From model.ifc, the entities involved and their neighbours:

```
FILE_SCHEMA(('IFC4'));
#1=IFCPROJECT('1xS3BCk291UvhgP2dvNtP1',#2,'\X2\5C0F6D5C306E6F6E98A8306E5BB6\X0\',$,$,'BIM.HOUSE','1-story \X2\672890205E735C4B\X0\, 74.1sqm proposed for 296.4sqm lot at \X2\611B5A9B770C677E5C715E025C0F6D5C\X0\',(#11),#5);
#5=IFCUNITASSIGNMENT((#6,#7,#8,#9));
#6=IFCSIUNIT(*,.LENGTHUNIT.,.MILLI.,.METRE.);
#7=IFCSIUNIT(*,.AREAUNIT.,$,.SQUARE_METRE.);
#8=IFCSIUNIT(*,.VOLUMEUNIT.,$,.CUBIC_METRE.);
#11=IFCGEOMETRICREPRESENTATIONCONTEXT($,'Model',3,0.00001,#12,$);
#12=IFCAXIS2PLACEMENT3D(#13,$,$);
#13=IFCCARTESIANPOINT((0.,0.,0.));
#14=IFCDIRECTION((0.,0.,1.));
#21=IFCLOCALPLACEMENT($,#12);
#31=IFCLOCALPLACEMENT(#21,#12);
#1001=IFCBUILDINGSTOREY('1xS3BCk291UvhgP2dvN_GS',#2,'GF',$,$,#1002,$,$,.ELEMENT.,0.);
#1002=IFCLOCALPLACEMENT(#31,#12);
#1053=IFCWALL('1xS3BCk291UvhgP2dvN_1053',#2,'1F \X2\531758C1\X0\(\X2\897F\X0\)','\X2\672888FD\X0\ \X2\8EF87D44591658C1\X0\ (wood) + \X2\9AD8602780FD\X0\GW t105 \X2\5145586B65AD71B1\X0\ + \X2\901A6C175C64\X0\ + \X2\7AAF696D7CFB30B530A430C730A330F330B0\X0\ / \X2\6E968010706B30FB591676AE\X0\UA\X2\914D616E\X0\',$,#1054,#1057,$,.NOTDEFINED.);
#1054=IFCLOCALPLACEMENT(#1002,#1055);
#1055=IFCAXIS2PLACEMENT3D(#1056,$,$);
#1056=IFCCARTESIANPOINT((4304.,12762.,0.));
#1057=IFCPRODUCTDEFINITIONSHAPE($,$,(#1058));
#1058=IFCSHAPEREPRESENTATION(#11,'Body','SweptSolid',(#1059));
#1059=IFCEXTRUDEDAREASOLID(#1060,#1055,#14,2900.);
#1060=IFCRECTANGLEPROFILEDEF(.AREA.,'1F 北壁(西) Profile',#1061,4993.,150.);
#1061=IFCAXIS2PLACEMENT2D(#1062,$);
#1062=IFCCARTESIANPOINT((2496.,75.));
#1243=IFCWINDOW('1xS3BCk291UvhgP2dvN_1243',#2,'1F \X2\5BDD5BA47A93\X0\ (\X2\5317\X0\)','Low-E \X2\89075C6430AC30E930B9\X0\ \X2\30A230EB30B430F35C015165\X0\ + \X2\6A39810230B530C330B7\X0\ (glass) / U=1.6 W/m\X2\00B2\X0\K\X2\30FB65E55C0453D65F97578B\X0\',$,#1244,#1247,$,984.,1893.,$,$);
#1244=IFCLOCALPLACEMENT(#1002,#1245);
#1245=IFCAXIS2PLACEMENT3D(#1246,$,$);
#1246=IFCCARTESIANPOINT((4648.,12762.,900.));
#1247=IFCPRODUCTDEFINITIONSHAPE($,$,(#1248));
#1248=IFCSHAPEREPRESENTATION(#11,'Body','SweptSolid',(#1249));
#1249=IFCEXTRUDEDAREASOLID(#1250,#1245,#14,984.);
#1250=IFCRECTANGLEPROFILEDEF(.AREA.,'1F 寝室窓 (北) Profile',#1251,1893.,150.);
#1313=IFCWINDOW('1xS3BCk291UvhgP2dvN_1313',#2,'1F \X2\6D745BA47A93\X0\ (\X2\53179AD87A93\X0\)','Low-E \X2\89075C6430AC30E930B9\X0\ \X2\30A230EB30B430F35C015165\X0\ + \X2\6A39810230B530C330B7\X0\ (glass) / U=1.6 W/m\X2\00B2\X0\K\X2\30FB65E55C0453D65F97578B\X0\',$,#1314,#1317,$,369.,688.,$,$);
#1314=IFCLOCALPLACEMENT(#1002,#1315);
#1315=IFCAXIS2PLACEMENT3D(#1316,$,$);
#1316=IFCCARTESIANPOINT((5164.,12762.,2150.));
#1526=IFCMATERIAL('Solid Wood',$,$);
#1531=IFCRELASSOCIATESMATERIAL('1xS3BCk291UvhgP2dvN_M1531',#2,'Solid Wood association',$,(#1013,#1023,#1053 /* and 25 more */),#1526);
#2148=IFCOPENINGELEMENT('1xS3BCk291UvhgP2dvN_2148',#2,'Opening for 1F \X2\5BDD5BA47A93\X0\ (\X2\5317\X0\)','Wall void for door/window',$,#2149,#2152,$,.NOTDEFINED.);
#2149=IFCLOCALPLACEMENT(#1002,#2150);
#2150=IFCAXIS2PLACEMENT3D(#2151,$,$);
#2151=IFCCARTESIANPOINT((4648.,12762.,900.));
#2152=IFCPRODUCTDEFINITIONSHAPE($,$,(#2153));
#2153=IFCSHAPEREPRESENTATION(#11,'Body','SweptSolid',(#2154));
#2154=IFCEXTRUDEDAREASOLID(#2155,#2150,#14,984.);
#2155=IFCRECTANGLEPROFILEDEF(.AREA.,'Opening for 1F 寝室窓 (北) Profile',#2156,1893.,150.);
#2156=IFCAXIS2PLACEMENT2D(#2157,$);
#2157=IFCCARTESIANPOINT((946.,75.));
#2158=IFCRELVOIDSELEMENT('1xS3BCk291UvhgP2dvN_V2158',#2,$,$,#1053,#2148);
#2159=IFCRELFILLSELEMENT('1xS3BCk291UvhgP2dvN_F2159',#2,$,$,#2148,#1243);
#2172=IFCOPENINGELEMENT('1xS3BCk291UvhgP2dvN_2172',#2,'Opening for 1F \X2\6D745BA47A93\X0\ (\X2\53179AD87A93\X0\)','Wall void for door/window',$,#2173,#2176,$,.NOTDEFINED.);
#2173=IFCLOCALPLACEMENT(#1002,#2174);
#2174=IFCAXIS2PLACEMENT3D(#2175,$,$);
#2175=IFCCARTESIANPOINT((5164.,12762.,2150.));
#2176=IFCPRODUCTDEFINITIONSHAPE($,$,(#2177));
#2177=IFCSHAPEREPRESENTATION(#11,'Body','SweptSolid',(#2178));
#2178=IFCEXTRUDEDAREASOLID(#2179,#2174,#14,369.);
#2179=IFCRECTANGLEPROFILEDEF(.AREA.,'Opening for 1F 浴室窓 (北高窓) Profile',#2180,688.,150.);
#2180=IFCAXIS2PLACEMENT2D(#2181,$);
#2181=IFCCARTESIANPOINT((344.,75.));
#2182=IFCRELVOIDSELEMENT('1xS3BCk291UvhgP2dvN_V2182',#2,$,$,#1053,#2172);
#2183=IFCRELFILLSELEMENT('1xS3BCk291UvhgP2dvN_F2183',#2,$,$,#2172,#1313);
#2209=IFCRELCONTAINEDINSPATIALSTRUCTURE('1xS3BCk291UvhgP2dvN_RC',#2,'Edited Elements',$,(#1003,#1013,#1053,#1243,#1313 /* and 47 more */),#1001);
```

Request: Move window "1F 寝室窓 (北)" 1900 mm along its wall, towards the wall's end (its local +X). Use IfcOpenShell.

```python
import ifcopenshell
import ifcopenshell.api.geometry
import ifcopenshell.util.placement

model = ifcopenshell.open("model.ifc")

window = model.by_id(1243)
opening = window.FillsVoids[0].RelatingOpeningElement
wall = opening.VoidsElements[0].RelatingBuildingElement

wall_matrix = ifcopenshell.util.placement.get_local_placement(wall.ObjectPlacement)
shift = wall_matrix[:3, 0] * 1900.0
before = ifcopenshell.util.placement.get_local_placement(window.ObjectPlacement)[:3, 3].copy()

# The window is not placed relative to its opening, so move both.
for product in (opening, window):
    matrix = ifcopenshell.util.placement.get_local_placement(product.ObjectPlacement)
    matrix[:3, 3] += shift
    ifcopenshell.api.geometry.edit_object_placement(model, product=product, matrix=matrix, is_si=False)

after = ifcopenshell.util.placement.get_local_placement(window.ObjectPlacement)[:3, 3]
print("window moved by", (after - before).round(3) + 0.0)

model.write("model_updated.ifc")
```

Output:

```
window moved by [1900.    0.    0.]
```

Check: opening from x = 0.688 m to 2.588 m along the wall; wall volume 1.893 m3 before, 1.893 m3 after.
